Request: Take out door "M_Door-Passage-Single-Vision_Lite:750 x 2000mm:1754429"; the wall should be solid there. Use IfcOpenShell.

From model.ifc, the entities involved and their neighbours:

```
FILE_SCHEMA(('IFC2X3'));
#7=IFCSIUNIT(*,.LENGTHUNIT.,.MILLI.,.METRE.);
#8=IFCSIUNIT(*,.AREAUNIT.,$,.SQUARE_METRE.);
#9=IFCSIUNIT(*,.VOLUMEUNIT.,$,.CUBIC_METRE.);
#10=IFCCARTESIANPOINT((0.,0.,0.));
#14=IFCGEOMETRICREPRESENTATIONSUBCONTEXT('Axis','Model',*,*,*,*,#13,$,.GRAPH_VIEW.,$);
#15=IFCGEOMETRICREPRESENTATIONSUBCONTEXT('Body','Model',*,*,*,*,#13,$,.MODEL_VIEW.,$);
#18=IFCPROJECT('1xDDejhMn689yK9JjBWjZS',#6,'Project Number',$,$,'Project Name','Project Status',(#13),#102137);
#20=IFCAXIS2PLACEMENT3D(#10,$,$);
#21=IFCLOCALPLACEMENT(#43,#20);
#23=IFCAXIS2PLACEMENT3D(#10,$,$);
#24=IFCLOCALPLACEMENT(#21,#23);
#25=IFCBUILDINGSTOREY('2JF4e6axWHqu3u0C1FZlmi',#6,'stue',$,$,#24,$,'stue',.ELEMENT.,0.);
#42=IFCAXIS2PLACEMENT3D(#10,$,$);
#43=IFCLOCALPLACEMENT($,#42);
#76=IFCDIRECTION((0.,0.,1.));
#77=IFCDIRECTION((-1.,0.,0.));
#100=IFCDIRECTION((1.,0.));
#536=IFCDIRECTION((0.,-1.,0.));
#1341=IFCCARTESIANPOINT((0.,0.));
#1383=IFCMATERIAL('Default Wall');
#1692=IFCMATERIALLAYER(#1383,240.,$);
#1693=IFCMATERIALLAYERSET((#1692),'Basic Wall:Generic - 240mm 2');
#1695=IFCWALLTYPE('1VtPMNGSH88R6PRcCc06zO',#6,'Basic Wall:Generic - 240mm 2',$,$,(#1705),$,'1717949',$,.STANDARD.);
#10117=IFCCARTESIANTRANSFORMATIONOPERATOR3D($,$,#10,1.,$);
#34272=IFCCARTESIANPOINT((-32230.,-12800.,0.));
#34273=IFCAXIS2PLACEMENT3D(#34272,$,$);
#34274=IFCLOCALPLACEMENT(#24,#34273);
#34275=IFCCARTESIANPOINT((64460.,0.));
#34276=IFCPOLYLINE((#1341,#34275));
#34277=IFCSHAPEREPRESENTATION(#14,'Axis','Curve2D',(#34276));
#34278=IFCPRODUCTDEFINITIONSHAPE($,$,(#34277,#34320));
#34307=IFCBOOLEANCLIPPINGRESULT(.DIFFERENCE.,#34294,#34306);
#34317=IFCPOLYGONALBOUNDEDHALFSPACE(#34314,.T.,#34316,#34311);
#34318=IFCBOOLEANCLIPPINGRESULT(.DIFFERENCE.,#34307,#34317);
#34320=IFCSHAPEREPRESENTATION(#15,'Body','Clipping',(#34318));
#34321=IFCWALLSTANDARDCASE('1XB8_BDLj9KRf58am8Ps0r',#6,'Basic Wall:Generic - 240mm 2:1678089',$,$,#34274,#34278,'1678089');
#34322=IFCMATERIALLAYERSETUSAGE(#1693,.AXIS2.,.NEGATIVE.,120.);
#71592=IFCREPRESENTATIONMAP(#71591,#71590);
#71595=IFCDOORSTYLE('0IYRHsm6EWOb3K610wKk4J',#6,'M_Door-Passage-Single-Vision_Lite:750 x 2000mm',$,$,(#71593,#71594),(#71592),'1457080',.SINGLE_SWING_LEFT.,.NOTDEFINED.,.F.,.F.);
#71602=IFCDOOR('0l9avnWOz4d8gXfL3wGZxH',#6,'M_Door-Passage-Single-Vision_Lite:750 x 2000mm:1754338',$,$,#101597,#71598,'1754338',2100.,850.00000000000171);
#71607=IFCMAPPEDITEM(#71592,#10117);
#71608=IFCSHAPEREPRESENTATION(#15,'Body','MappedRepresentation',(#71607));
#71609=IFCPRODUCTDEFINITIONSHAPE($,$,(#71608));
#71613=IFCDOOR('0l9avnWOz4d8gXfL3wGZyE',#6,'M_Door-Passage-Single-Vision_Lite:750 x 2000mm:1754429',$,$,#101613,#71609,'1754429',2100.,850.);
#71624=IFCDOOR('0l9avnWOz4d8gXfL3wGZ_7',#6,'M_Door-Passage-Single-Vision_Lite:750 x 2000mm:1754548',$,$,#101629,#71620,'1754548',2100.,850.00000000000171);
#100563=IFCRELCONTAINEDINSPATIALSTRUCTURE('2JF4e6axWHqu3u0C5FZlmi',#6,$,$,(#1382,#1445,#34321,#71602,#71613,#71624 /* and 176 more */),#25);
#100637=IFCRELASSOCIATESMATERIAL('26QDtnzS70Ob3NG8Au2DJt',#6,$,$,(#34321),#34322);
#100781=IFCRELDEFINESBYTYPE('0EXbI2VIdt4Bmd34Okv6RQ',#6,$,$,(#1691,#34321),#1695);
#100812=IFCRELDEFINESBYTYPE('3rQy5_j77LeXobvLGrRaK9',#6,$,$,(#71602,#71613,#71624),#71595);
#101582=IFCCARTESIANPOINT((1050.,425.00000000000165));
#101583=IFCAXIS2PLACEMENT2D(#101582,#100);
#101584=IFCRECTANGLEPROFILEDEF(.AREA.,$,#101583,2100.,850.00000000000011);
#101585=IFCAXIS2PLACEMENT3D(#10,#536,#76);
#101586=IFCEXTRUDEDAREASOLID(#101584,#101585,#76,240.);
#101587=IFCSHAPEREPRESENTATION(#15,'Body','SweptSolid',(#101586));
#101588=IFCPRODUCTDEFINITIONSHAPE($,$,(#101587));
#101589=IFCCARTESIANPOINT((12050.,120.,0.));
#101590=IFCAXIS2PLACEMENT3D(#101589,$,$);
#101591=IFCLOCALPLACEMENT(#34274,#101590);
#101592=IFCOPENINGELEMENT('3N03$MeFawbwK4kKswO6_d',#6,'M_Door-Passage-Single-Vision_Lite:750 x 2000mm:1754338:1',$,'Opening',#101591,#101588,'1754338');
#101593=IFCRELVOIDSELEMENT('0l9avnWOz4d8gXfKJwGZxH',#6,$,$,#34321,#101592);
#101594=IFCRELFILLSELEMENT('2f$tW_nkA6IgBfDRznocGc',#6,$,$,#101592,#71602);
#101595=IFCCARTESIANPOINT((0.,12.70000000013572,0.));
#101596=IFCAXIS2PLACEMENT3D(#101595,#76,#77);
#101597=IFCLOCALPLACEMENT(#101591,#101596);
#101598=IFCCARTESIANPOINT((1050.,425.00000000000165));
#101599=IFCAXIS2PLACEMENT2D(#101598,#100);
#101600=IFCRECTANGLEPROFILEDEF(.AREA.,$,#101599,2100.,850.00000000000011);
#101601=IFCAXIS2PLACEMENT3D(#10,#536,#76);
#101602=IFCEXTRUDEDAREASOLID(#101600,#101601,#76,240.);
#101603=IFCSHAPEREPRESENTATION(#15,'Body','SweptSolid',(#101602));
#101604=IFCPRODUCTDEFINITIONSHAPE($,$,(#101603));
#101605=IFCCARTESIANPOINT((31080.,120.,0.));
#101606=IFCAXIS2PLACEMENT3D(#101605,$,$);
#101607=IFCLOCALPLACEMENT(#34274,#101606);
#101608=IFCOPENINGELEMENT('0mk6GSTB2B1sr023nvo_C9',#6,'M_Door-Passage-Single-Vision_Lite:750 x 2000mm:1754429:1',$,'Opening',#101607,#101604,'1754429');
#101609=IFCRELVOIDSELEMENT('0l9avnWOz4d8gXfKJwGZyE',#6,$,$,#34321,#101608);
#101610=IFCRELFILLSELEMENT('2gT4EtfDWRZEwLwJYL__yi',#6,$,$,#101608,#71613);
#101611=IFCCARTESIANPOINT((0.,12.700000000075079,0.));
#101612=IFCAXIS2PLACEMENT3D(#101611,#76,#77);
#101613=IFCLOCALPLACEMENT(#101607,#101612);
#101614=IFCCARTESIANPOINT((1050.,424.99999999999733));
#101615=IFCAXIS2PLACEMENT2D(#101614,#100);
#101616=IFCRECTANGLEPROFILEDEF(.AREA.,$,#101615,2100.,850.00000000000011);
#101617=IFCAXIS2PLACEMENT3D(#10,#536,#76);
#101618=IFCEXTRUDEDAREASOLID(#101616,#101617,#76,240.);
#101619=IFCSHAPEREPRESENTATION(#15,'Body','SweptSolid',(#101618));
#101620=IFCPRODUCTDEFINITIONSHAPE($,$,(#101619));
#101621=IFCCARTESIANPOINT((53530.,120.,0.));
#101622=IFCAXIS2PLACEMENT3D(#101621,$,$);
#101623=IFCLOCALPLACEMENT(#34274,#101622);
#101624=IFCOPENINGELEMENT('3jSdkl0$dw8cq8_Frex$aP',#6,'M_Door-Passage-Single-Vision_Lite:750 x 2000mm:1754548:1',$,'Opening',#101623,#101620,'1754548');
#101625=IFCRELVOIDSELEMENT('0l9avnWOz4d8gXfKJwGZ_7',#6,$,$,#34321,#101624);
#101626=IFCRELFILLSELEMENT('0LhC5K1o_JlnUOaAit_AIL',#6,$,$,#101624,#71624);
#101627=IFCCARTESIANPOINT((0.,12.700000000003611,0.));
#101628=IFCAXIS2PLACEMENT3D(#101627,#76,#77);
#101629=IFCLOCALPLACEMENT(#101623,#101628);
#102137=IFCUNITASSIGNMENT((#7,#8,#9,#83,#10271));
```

```python
import ifcopenshell
import ifcopenshell.api.feature
import ifcopenshell.api.root
import ifcopenshell.geom
import ifcopenshell.util.shape

model = ifcopenshell.open("model.ifc")
settings = ifcopenshell.geom.settings()


def volume(element):
    """Net volume in cubic metres, openings subtracted."""
    shape = ifcopenshell.geom.create_shape(settings, element)
    return ifcopenshell.util.shape.get_volume(shape.geometry)


door = model.by_guid("0l9avnWOz4d8gXfL3wGZyE")
opening = door.FillsVoids[0].RelatingOpeningElement
wall = opening.VoidsElements[0].RelatingBuildingElement
before = volume(wall)

ifcopenshell.api.root.remove_product(model, product=door)
ifcopenshell.api.feature.remove_feature(model, feature=opening)

after = volume(wall)

print(f"wall volume {before:.3f} -> {after:.3f} m3")

model.write("model_v2.ifc")
```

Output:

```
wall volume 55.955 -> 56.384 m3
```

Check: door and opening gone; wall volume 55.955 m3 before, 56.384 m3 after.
